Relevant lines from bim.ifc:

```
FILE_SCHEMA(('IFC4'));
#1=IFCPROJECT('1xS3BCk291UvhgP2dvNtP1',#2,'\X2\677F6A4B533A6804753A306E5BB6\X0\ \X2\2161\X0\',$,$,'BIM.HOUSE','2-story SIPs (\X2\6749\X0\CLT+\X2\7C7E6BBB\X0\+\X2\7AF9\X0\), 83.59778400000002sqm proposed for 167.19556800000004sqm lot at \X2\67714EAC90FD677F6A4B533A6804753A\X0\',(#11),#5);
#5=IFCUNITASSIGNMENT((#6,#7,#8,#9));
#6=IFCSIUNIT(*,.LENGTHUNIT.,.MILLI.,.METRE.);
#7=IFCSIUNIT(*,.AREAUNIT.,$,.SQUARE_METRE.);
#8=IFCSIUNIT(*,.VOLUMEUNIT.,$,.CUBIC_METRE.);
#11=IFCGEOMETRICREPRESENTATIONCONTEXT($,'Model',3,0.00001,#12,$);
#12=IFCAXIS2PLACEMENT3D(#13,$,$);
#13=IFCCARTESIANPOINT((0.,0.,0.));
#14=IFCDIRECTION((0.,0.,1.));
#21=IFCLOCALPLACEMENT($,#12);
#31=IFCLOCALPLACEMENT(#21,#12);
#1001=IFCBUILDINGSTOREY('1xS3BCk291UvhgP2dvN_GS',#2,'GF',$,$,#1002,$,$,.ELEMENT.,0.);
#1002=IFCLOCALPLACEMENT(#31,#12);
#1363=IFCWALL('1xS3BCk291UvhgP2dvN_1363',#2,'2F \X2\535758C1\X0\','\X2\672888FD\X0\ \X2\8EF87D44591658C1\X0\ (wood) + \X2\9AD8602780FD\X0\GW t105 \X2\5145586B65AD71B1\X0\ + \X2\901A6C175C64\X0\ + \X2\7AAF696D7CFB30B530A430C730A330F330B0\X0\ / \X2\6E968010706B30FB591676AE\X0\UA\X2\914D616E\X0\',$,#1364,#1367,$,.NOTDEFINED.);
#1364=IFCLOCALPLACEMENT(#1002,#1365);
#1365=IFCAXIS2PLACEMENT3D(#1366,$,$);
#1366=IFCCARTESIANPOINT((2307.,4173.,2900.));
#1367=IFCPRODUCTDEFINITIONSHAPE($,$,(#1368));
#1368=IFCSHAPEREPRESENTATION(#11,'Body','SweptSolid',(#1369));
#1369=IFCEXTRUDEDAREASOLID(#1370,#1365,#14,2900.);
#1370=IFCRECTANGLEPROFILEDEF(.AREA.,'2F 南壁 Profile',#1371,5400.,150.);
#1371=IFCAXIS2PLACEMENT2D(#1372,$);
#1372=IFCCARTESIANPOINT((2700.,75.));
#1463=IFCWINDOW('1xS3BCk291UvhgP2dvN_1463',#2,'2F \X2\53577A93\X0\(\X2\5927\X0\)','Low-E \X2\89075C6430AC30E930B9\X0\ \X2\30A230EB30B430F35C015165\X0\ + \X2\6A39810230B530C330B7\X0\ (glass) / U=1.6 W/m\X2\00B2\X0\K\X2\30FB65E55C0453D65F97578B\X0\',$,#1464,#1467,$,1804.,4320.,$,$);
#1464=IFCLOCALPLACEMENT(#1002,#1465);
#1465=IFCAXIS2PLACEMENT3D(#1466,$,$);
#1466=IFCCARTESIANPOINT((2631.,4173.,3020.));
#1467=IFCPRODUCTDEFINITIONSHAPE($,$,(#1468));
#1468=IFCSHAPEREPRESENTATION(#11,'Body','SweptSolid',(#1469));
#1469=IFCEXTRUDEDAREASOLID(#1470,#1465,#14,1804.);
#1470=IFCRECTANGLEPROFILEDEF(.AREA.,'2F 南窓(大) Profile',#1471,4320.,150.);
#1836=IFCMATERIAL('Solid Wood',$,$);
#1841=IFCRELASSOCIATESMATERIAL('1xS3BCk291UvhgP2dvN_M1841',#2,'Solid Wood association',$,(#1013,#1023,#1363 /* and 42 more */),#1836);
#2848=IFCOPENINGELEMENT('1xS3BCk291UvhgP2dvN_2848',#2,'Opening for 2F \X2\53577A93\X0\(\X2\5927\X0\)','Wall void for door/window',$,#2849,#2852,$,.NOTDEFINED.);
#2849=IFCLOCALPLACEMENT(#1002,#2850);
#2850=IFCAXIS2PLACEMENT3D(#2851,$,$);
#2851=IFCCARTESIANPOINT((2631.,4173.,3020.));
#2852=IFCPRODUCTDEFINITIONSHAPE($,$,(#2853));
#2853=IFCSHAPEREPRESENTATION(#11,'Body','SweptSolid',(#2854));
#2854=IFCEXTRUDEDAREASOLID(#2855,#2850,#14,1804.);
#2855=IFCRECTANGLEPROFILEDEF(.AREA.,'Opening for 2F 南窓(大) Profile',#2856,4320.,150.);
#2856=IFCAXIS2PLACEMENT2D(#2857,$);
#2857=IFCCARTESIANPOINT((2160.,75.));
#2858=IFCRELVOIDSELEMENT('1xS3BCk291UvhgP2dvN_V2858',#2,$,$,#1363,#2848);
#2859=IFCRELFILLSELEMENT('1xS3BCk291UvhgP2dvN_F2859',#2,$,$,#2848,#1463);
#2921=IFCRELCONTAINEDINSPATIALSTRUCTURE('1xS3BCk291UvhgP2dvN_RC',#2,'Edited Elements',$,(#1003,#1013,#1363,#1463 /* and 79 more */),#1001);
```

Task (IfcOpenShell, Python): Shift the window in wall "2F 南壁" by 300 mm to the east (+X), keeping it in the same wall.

```python
import ifcopenshell
import ifcopenshell.api.geometry
import ifcopenshell.util.placement
import ifcopenshell.util.unit

model = ifcopenshell.open("bim.ifc")
unit_scale = ifcopenshell.util.unit.calculate_unit_scale(model)

window = model.by_guid("1xS3BCk291UvhgP2dvN_1463")
opening = window.FillsVoids[0].RelatingOpeningElement
wall = opening.VoidsElements[0].RelatingBuildingElement

wall_matrix = ifcopenshell.util.placement.get_local_placement(wall.ObjectPlacement)
shift = wall_matrix[:3, 0] * 0.3 / unit_scale
before = ifcopenshell.util.placement.get_local_placement(window.ObjectPlacement)[:3, 3].copy()

# The window is not placed relative to its opening, so move both.
for product in (opening, window):
    matrix = ifcopenshell.util.placement.get_local_placement(product.ObjectPlacement)
    matrix[:3, 3] += shift
    ifcopenshell.api.geometry.edit_object_placement(model, product=product, matrix=matrix, is_si=False)

after = ifcopenshell.util.placement.get_local_placement(window.ObjectPlacement)[:3, 3]
print("window moved by", (after - before).round(3) + 0.0)

model.write("bim_updated.ifc")
```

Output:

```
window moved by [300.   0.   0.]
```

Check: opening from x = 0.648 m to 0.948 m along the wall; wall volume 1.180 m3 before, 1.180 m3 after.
